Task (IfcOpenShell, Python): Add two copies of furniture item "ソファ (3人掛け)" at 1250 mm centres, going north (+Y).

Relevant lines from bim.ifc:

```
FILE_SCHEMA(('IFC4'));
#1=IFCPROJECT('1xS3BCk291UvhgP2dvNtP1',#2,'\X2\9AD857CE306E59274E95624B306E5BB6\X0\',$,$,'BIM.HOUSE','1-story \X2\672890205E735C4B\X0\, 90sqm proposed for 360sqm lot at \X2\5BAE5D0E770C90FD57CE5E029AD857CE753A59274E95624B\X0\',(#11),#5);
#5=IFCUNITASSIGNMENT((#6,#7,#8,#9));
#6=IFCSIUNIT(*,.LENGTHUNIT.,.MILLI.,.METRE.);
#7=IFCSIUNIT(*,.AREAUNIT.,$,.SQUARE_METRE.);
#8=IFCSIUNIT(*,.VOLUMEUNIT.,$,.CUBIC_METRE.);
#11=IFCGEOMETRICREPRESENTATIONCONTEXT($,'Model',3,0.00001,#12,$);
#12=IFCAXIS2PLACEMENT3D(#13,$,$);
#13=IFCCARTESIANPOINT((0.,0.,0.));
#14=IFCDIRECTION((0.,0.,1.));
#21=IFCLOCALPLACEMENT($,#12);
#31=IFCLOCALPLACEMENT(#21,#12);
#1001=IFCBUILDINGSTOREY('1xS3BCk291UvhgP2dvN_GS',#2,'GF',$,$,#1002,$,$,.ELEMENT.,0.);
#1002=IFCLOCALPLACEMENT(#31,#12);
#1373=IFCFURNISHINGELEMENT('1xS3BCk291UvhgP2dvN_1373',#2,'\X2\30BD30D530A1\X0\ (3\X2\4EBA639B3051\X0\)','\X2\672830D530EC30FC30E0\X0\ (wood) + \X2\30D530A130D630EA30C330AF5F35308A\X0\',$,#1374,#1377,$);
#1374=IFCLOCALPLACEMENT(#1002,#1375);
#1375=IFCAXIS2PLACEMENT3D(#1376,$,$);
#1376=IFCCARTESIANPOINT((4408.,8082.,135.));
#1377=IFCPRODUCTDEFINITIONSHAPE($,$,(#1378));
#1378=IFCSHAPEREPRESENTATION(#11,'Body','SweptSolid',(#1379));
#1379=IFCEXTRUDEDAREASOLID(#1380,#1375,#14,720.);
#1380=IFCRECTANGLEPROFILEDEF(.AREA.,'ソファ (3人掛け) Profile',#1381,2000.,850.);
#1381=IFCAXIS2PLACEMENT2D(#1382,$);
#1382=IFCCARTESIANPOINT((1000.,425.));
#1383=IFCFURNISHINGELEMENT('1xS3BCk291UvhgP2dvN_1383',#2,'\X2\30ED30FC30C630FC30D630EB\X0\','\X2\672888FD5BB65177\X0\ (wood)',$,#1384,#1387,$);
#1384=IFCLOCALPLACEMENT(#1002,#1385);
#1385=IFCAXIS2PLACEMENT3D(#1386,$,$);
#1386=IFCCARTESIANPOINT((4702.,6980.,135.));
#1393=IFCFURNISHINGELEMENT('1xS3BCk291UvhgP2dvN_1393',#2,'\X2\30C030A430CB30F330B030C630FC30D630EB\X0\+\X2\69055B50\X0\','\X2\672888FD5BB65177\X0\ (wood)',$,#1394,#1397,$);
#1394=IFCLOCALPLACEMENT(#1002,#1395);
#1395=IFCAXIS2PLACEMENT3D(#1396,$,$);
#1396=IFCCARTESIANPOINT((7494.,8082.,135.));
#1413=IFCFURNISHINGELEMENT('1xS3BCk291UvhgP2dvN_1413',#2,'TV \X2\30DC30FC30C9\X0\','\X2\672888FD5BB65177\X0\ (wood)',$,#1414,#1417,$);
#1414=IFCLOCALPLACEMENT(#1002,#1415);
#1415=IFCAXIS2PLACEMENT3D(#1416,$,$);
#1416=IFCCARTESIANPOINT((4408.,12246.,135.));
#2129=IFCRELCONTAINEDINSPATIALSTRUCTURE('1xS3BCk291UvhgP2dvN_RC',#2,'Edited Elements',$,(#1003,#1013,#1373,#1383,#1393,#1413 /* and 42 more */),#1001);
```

```python
import numpy as np
import ifcopenshell
import ifcopenshell.api.geometry
import ifcopenshell.api.root
import ifcopenshell.util.element
import ifcopenshell.util.placement
import ifcopenshell.util.unit

model = ifcopenshell.open("bim.ifc")
unit_scale = ifcopenshell.util.unit.calculate_unit_scale(model)


def reuse_history(source, copy):
    """copy_class also copies each property set's owner history, people and application; keep the originals."""
    for rel in copy.IsDefinedBy:
        if rel.is_a("IfcRelDefinesByProperties") and (history := rel.RelatingPropertyDefinition.OwnerHistory):
            rel.RelatingPropertyDefinition.OwnerHistory = source.OwnerHistory
            ifcopenshell.util.element.remove_deep2(model, history)


source = model.by_id(1373)
base = ifcopenshell.util.placement.get_local_placement(source.ObjectPlacement)
step = np.array([0.0, 1.0, 0.0]) * 1.25 / unit_scale

for i in range(1, 3):
    copy = ifcopenshell.api.root.copy_class(model, product=source)
    copy.Representation = ifcopenshell.util.element.copy_deep(
        model, source.Representation, exclude=["IfcGeometricRepresentationContext", "IfcRepresentationMap"]
    )
    reuse_history(source, copy)
    matrix = base.copy()
    matrix[:3, 3] += i * step
    print("added at", matrix[:3, 3].round(3) + 0.0)
    ifcopenshell.api.geometry.edit_object_placement(model, product=copy, matrix=matrix, is_si=False)

model.write("bim_rev.ifc")
```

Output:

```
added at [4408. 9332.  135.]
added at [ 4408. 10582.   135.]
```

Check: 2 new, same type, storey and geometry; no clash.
